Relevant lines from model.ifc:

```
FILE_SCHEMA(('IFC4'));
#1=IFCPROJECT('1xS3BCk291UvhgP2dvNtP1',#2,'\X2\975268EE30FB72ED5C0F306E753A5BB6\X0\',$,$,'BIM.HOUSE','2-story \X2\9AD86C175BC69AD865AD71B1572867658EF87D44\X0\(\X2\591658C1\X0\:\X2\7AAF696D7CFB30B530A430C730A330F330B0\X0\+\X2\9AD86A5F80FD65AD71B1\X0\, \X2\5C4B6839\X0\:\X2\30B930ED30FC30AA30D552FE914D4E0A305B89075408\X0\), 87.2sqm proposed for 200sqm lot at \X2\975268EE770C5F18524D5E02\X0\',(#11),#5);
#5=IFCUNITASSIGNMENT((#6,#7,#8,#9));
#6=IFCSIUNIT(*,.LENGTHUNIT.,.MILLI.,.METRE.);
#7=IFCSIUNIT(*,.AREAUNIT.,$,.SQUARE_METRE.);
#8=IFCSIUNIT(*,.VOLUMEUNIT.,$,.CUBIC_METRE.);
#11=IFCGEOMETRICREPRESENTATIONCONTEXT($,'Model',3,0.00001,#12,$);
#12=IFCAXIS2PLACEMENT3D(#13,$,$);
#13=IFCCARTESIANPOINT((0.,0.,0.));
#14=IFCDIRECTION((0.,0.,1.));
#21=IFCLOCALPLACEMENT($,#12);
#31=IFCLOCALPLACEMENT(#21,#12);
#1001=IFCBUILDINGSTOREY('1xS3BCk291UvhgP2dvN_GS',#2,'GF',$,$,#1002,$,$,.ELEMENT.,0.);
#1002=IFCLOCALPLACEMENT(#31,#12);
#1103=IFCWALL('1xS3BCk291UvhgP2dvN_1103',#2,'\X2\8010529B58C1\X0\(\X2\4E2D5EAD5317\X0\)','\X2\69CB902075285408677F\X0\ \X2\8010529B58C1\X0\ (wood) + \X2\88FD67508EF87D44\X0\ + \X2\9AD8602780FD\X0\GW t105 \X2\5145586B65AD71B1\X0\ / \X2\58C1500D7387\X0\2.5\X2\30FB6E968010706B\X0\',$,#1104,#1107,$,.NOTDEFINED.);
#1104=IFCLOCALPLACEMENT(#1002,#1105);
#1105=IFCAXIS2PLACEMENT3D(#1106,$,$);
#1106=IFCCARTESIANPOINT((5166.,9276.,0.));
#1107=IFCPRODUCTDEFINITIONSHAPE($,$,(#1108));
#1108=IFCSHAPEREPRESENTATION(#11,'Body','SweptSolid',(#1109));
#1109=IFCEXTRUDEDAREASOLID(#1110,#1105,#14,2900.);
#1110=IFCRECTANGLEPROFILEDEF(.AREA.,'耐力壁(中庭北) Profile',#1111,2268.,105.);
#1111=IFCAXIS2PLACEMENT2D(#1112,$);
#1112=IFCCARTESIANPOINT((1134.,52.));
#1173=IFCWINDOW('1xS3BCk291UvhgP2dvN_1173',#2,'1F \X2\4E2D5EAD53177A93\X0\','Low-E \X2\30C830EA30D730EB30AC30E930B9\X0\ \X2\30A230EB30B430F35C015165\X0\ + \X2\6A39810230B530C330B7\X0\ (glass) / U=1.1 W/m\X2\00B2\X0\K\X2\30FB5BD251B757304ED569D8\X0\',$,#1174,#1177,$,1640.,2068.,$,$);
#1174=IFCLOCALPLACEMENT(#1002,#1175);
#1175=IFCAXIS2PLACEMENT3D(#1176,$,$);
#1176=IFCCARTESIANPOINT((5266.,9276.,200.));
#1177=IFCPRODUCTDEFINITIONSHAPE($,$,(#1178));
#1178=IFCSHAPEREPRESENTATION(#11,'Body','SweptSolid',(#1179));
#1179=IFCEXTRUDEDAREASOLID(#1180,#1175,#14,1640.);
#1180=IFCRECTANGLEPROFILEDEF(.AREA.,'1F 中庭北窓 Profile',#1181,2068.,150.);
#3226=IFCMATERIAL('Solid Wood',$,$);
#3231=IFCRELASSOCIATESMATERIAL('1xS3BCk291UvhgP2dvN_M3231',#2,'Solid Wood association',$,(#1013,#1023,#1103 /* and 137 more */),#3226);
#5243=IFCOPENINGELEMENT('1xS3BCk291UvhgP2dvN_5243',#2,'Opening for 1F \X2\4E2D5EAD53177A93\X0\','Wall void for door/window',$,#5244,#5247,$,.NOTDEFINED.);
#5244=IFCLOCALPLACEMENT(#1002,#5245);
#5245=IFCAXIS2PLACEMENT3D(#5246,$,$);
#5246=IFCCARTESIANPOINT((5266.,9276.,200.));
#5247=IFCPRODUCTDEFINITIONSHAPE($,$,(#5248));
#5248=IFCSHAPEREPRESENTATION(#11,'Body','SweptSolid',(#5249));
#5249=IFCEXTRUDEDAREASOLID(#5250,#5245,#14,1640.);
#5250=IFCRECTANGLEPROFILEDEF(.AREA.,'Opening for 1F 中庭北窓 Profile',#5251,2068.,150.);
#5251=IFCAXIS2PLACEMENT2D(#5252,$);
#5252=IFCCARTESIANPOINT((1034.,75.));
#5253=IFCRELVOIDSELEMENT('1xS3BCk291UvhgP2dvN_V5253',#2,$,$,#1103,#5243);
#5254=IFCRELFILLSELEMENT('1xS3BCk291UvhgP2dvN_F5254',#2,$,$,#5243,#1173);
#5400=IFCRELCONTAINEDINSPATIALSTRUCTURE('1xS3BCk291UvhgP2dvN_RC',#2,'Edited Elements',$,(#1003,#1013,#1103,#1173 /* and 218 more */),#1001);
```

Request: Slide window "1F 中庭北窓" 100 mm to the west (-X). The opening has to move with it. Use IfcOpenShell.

```python
import ifcopenshell
import ifcopenshell.api.geometry
import ifcopenshell.util.placement
import ifcopenshell.util.unit

model = ifcopenshell.open("model.ifc")
unit_scale = ifcopenshell.util.unit.calculate_unit_scale(model)

window = model.by_guid("1xS3BCk291UvhgP2dvN_1173")
opening = window.FillsVoids[0].RelatingOpeningElement
wall = opening.VoidsElements[0].RelatingBuildingElement

wall_matrix = ifcopenshell.util.placement.get_local_placement(wall.ObjectPlacement)
shift = wall_matrix[:3, 0] * -0.1 / unit_scale
before = ifcopenshell.util.placement.get_local_placement(window.ObjectPlacement)[:3, 3].copy()

# The window is not placed relative to its opening, so move both.
for product in (opening, window):
    matrix = ifcopenshell.util.placement.get_local_placement(product.ObjectPlacement)
    matrix[:3, 3] += shift
    ifcopenshell.api.geometry.edit_object_placement(model, product=product, matrix=matrix, is_si=False)

after = ifcopenshell.util.placement.get_local_placement(window.ObjectPlacement)[:3, 3]
print("window moved by", (after - before).round(3) + 0.0)

model.write("model_rev.ifc")
```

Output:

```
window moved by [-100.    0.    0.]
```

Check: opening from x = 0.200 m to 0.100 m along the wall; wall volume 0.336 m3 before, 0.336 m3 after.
